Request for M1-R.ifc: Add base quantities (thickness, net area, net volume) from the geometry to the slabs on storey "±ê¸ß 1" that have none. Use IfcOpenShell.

First a look at what the model holds.

```python
import ifcopenshell
import ifcopenshell.util.element
import ifcopenshell.util.unit

model = ifcopenshell.open("M1-R.ifc")
print(model.schema)
for unit_type in ("LENGTHUNIT", "AREAUNIT", "VOLUMEUNIT"):
    print(unit_type, ifcopenshell.util.unit.calculate_unit_scale(model, unit_type))
storey = next(s for s in model.by_type("IfcBuildingStorey") if s.Name == "±ê¸ß 1")
slabs = [e for e in ifcopenshell.util.element.get_decomposition(storey) if e.is_a("IfcSlab")]
for e in sorted(slabs, key=lambda e: e.id()):
    print(e.id(), e.is_a(), e.Name, list(ifcopenshell.util.element.get_psets(e, qtos_only=True)), sep=" | ")
```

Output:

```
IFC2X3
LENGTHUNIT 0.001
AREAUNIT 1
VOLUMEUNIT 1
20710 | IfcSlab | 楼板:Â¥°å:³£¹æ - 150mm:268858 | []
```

```python
import ifcopenshell
import ifcopenshell.api.pset
import ifcopenshell.geom
import ifcopenshell.util.element
import ifcopenshell.util.shape
import ifcopenshell.util.unit

model = ifcopenshell.open("M1-R.ifc")
unit_scale = ifcopenshell.util.unit.calculate_unit_scale(model)
area_scale = ifcopenshell.util.unit.calculate_unit_scale(model, "AREAUNIT")
volume_scale = ifcopenshell.util.unit.calculate_unit_scale(model, "VOLUMEUNIT")
settings = ifcopenshell.geom.settings()

storey = next(s for s in model.by_type("IfcBuildingStorey") if s.Name == "±ê¸ß 1")
slabs = [e for e in ifcopenshell.util.element.get_decomposition(storey) if e.is_a("IfcSlab")]

for e in sorted(slabs, key=lambda e: e.id()):
    if ifcopenshell.util.element.get_psets(e, qtos_only=True, should_inherit=False):
        continue
    # Geometry comes back in metres, in the element's own axes.
    shape = ifcopenshell.geom.create_shape(settings, e)
    values = {
        "Width": ifcopenshell.util.shape.get_z(shape.geometry) / unit_scale,
        "NetArea": ifcopenshell.util.shape.get_footprint_area(shape.geometry) / area_scale,
        "NetVolume": ifcopenshell.util.shape.get_volume(shape.geometry) / volume_scale,
    }
    qto = ifcopenshell.api.pset.add_qto(model, product=e, name="BaseQuantities")
    ifcopenshell.api.pset.edit_qto(model, qto=qto, properties=values)
    print(e.id(), {k: round(v, 3) for k, v in values.items()})

model.write("M1-R-out.ifc")
```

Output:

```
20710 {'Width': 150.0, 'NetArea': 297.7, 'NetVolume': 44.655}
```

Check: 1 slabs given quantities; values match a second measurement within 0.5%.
